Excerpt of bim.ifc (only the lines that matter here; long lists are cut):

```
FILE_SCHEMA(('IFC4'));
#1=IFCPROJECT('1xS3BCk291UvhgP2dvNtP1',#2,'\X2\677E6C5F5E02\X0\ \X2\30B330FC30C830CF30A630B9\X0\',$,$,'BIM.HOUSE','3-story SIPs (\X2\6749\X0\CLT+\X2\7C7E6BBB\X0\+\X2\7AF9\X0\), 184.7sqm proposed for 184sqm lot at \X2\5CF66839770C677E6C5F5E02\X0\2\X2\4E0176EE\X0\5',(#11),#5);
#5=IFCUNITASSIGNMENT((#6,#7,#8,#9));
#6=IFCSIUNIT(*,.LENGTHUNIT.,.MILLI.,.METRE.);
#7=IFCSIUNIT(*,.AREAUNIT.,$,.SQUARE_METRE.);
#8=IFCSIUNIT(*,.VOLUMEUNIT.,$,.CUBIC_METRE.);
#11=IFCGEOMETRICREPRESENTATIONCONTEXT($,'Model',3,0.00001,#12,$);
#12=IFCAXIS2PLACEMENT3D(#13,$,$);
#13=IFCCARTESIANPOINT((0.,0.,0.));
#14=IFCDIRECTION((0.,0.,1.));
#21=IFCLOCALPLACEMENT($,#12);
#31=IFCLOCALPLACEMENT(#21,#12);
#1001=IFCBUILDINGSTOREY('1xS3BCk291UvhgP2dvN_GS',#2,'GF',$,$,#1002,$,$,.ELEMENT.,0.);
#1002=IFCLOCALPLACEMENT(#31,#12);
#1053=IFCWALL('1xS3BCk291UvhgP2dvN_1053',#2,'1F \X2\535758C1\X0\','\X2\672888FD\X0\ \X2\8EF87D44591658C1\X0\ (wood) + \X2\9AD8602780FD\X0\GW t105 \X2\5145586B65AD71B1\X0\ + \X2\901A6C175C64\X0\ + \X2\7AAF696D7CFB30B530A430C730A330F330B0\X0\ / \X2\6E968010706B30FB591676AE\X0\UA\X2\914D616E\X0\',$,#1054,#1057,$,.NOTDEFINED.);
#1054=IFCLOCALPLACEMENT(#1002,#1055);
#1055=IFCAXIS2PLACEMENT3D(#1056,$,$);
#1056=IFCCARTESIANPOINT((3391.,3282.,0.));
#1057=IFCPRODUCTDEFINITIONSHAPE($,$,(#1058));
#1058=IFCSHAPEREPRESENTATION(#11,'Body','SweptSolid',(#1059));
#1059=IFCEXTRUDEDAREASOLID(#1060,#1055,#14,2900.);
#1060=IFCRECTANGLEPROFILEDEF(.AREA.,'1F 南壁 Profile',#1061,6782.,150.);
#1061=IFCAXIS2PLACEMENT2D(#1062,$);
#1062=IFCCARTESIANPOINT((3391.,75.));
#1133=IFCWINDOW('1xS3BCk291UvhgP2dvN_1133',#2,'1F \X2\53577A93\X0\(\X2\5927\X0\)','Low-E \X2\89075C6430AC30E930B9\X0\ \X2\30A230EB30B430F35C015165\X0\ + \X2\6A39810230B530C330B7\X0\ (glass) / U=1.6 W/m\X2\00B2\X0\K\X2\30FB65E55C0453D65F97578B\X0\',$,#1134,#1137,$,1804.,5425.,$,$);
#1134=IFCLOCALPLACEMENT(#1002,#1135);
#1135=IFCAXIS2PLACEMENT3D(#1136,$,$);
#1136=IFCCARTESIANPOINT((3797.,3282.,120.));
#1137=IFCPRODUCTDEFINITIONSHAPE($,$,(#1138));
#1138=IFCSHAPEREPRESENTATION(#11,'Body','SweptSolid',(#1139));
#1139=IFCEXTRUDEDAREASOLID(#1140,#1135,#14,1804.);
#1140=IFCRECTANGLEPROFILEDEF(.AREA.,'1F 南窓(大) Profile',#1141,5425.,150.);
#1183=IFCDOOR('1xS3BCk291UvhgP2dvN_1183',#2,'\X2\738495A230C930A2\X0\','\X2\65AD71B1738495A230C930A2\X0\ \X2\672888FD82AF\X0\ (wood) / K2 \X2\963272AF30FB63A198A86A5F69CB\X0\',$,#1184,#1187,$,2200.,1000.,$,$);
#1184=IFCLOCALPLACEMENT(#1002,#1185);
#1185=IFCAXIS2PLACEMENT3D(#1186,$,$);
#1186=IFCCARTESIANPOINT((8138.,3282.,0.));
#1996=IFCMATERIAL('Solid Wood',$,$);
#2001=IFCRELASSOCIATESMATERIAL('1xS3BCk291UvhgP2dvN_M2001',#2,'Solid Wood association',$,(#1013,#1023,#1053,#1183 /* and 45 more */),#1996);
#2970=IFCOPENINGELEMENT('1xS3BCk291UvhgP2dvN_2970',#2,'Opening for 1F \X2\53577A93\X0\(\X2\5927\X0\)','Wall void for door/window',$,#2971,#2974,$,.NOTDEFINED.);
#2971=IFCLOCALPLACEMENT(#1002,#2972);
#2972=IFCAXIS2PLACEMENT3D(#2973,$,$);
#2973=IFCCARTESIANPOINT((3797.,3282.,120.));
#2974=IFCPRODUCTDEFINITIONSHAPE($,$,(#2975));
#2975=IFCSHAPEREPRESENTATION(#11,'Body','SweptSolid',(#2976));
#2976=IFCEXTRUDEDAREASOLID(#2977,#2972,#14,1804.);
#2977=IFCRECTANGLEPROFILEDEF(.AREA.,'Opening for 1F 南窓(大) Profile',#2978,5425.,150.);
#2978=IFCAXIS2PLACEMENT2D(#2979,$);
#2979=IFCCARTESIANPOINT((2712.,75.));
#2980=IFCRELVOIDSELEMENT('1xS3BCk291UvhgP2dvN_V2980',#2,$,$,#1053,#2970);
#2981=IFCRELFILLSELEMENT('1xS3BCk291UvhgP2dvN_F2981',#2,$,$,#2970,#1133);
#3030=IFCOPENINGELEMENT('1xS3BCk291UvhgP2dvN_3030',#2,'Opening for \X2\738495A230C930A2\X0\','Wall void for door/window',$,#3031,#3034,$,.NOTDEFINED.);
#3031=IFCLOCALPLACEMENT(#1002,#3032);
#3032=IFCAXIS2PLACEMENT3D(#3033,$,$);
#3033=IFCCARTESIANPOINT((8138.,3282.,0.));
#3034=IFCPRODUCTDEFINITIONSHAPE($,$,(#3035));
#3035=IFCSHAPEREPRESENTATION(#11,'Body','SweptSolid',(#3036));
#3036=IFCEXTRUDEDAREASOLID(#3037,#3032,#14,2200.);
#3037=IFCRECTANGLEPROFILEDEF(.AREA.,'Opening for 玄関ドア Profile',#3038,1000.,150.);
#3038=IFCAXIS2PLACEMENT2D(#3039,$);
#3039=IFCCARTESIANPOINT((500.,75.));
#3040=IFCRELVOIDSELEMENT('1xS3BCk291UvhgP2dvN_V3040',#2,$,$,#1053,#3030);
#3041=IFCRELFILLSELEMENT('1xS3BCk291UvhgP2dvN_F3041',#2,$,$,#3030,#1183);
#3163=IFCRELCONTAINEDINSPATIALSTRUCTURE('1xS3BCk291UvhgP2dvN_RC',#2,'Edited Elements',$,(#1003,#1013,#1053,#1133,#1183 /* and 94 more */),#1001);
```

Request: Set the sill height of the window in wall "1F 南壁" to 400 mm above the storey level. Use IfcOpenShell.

```python
import numpy as np
import ifcopenshell
import ifcopenshell.api.geometry
import ifcopenshell.geom
import ifcopenshell.util.element
import ifcopenshell.util.placement
import ifcopenshell.util.shape
import ifcopenshell.util.unit

model = ifcopenshell.open("bim.ifc")
unit_scale = ifcopenshell.util.unit.calculate_unit_scale(model)

window = model.by_guid("1xS3BCk291UvhgP2dvN_1133")
opening = window.FillsVoids[0].RelatingOpeningElement
storey = ifcopenshell.util.element.get_container(window, ifc_class="IfcBuildingStorey")
level = ifcopenshell.util.placement.get_local_placement(storey.ObjectPlacement)[2, 3]

# The opening's origin need not be at the sill, so measure its lowest point.
shape = ifcopenshell.geom.create_shape(ifcopenshell.geom.settings(), opening)
bottom = ifcopenshell.util.shape.get_shape_bottom_elevation(shape, shape.geometry) / unit_scale
dz = level + 400.0 - bottom

shift = np.array([0.0, 0.0, dz])
# The window is not placed relative to its opening, so move both.
for product in (opening, window):
    matrix = ifcopenshell.util.placement.get_local_placement(product.ObjectPlacement)
    matrix[:3, 3] += shift
    ifcopenshell.api.geometry.edit_object_placement(model, product=product, matrix=matrix, is_si=False)

print(f"moved by {dz * unit_scale:+.3f} m")

model.write("bim-out.ifc")
```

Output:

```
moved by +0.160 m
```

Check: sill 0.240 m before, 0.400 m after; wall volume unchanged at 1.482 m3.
